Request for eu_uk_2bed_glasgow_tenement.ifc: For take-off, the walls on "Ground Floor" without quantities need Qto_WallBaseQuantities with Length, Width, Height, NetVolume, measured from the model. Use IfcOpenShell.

First a look at what the model holds.

```python
import ifcopenshell
import ifcopenshell.util.element
import ifcopenshell.util.unit

model = ifcopenshell.open("eu_uk_2bed_glasgow_tenement.ifc")
print(model.schema)
for unit_type in ("LENGTHUNIT", "AREAUNIT", "VOLUMEUNIT"):
    print(unit_type, ifcopenshell.util.unit.calculate_unit_scale(model, unit_type))
storey = next(s for s in model.by_type("IfcBuildingStorey") if s.Name == "Ground Floor")
walls = [e for e in ifcopenshell.util.element.get_decomposition(storey) if e.is_a("IfcWall")]
for e in sorted(walls, key=lambda e: e.id()):
    print(e.id(), e.is_a(), e.Name, list(ifcopenshell.util.element.get_psets(e, qtos_only=True)), sep=" | ")
```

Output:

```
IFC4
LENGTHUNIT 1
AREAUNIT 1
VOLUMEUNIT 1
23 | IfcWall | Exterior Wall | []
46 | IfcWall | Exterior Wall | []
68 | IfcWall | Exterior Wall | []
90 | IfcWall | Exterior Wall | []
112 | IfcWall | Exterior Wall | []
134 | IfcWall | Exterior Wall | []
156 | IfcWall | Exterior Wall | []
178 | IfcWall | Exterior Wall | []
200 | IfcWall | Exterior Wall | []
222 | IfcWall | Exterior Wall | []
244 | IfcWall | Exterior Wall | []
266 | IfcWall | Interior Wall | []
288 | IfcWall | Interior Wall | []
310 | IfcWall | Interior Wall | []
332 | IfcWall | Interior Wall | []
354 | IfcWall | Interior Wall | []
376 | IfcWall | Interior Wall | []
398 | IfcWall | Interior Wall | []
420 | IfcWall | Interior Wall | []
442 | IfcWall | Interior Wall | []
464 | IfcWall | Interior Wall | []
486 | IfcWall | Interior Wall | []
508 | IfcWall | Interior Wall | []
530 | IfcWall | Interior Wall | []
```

```python
import ifcopenshell
import ifcopenshell.api.pset
import ifcopenshell.geom
import ifcopenshell.util.element
import ifcopenshell.util.shape
import ifcopenshell.util.unit

model = ifcopenshell.open("eu_uk_2bed_glasgow_tenement.ifc")
unit_scale = ifcopenshell.util.unit.calculate_unit_scale(model)
volume_scale = ifcopenshell.util.unit.calculate_unit_scale(model, "VOLUMEUNIT")
settings = ifcopenshell.geom.settings()

storey = next(s for s in model.by_type("IfcBuildingStorey") if s.Name == "Ground Floor")
walls = [e for e in ifcopenshell.util.element.get_decomposition(storey) if e.is_a("IfcWall")]

for e in sorted(walls, key=lambda e: e.id()):
    if ifcopenshell.util.element.get_psets(e, qtos_only=True, should_inherit=False):
        continue
    # Geometry comes back in metres, in the element's own axes.
    shape = ifcopenshell.geom.create_shape(settings, e)
    values = {
        "Length": ifcopenshell.util.shape.get_x(shape.geometry) / unit_scale,
        "Width": ifcopenshell.util.shape.get_y(shape.geometry) / unit_scale,
        "Height": ifcopenshell.util.shape.get_z(shape.geometry) / unit_scale,
        "NetVolume": ifcopenshell.util.shape.get_volume(shape.geometry) / volume_scale,
    }
    qto = ifcopenshell.api.pset.add_qto(model, product=e, name="Qto_WallBaseQuantities")
    ifcopenshell.api.pset.edit_qto(model, qto=qto, properties=values)
    print(e.id(), {k: round(v, 3) for k, v in values.items()})

model.write("eu_uk_2bed_glasgow_tenement-out.ifc")
```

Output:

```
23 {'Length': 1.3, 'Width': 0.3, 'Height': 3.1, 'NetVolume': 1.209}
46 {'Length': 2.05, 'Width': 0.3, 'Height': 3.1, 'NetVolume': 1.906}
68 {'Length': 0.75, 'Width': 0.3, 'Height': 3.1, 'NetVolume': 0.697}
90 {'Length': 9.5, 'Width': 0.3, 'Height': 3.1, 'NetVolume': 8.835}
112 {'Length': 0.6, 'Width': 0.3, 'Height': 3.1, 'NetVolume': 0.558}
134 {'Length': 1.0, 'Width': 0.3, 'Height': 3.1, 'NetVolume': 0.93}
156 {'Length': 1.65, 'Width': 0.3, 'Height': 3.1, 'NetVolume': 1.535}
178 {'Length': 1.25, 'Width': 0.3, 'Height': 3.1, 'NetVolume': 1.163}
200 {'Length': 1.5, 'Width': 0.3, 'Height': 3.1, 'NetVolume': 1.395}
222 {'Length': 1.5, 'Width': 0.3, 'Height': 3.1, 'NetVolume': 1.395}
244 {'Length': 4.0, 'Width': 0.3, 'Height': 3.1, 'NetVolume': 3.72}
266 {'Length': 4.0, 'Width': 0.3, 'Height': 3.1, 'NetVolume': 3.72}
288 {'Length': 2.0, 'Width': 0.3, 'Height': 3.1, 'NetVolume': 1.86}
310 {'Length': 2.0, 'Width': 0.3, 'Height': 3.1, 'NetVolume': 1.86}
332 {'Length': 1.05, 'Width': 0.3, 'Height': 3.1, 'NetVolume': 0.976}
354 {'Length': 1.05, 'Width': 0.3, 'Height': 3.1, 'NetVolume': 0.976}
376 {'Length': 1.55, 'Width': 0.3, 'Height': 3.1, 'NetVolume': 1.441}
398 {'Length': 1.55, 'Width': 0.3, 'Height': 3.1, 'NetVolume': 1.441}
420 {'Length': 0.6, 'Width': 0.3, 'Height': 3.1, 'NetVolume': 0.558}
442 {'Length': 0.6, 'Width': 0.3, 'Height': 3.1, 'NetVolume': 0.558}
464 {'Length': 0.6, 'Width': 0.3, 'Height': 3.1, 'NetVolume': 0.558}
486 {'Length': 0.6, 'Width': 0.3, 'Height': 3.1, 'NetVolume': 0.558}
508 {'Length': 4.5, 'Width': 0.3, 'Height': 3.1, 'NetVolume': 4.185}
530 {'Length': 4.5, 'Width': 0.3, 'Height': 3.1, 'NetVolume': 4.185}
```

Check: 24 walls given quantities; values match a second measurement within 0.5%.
